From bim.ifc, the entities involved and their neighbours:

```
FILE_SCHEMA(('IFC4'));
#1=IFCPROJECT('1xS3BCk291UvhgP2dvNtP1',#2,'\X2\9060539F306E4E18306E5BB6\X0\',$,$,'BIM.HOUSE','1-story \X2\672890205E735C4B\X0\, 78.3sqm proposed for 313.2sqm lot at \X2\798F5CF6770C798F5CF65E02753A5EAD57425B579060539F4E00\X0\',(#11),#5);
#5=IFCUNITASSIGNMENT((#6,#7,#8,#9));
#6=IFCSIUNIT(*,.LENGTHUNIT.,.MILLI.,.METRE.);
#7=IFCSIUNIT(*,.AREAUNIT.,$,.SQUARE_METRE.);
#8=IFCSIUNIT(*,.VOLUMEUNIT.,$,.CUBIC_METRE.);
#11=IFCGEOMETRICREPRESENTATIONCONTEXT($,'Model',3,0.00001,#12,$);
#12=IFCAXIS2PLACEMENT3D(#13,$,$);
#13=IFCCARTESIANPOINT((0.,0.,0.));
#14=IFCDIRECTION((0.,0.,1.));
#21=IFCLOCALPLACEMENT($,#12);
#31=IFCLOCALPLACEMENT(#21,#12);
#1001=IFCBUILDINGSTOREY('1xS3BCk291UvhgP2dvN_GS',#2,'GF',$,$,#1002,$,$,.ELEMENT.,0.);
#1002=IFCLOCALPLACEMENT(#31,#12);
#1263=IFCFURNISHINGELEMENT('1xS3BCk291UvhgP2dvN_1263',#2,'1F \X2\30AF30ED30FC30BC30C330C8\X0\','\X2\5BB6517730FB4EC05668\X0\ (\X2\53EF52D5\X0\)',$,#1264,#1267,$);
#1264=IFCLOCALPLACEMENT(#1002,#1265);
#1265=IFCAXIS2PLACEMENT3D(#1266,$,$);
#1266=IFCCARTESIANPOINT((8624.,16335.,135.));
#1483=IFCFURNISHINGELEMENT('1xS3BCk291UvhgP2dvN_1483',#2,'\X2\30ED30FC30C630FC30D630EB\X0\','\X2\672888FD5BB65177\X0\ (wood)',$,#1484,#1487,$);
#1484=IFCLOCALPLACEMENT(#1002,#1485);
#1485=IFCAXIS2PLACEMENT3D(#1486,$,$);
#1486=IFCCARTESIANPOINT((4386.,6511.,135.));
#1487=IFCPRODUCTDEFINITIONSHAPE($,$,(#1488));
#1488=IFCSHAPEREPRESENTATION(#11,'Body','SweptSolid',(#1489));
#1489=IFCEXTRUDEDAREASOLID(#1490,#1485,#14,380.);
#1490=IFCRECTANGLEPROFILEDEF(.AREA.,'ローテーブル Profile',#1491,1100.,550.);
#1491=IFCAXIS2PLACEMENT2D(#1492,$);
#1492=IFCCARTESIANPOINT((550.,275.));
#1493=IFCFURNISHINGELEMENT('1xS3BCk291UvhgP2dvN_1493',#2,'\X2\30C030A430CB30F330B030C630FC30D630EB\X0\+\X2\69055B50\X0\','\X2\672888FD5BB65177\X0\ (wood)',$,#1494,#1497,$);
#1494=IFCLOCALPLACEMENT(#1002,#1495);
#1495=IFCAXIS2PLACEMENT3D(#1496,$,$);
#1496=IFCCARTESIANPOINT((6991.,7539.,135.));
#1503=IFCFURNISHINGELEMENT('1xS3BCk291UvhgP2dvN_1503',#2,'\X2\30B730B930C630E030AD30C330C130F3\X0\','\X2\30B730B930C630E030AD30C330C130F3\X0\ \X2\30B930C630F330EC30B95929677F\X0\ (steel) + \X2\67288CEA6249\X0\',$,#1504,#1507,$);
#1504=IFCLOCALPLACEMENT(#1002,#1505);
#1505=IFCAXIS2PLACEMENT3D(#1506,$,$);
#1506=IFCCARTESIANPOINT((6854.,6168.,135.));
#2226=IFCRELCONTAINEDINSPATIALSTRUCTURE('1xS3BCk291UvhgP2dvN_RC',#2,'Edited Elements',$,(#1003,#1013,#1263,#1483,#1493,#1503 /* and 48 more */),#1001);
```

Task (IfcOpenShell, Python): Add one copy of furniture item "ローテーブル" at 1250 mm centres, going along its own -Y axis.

```python
import ifcopenshell
import ifcopenshell.api.geometry
import ifcopenshell.api.root
import ifcopenshell.util.element
import ifcopenshell.util.placement

model = ifcopenshell.open("bim.ifc")


def reuse_history(source, copy):
    """copy_class also copies each property set's owner history, people and application; keep the originals."""
    for rel in copy.IsDefinedBy:
        if rel.is_a("IfcRelDefinesByProperties") and (history := rel.RelatingPropertyDefinition.OwnerHistory):
            rel.RelatingPropertyDefinition.OwnerHistory = source.OwnerHistory
            ifcopenshell.util.element.remove_deep2(model, history)


source = model.by_id(1483)
base = ifcopenshell.util.placement.get_local_placement(source.ObjectPlacement)
step = -base[:3, 1] * 1250.0

for i in range(1, 2):
    copy = ifcopenshell.api.root.copy_class(model, product=source)
    copy.Representation = ifcopenshell.util.element.copy_deep(
        model, source.Representation, exclude=["IfcGeometricRepresentationContext", "IfcRepresentationMap"]
    )
    reuse_history(source, copy)
    matrix = base.copy()
    matrix[:3, 3] += i * step
    print("added at", matrix[:3, 3].round(3) + 0.0)
    ifcopenshell.api.geometry.edit_object_placement(model, product=copy, matrix=matrix, is_si=False)

model.write("bim_edited.ifc")
```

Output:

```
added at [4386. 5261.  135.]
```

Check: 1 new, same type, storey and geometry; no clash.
